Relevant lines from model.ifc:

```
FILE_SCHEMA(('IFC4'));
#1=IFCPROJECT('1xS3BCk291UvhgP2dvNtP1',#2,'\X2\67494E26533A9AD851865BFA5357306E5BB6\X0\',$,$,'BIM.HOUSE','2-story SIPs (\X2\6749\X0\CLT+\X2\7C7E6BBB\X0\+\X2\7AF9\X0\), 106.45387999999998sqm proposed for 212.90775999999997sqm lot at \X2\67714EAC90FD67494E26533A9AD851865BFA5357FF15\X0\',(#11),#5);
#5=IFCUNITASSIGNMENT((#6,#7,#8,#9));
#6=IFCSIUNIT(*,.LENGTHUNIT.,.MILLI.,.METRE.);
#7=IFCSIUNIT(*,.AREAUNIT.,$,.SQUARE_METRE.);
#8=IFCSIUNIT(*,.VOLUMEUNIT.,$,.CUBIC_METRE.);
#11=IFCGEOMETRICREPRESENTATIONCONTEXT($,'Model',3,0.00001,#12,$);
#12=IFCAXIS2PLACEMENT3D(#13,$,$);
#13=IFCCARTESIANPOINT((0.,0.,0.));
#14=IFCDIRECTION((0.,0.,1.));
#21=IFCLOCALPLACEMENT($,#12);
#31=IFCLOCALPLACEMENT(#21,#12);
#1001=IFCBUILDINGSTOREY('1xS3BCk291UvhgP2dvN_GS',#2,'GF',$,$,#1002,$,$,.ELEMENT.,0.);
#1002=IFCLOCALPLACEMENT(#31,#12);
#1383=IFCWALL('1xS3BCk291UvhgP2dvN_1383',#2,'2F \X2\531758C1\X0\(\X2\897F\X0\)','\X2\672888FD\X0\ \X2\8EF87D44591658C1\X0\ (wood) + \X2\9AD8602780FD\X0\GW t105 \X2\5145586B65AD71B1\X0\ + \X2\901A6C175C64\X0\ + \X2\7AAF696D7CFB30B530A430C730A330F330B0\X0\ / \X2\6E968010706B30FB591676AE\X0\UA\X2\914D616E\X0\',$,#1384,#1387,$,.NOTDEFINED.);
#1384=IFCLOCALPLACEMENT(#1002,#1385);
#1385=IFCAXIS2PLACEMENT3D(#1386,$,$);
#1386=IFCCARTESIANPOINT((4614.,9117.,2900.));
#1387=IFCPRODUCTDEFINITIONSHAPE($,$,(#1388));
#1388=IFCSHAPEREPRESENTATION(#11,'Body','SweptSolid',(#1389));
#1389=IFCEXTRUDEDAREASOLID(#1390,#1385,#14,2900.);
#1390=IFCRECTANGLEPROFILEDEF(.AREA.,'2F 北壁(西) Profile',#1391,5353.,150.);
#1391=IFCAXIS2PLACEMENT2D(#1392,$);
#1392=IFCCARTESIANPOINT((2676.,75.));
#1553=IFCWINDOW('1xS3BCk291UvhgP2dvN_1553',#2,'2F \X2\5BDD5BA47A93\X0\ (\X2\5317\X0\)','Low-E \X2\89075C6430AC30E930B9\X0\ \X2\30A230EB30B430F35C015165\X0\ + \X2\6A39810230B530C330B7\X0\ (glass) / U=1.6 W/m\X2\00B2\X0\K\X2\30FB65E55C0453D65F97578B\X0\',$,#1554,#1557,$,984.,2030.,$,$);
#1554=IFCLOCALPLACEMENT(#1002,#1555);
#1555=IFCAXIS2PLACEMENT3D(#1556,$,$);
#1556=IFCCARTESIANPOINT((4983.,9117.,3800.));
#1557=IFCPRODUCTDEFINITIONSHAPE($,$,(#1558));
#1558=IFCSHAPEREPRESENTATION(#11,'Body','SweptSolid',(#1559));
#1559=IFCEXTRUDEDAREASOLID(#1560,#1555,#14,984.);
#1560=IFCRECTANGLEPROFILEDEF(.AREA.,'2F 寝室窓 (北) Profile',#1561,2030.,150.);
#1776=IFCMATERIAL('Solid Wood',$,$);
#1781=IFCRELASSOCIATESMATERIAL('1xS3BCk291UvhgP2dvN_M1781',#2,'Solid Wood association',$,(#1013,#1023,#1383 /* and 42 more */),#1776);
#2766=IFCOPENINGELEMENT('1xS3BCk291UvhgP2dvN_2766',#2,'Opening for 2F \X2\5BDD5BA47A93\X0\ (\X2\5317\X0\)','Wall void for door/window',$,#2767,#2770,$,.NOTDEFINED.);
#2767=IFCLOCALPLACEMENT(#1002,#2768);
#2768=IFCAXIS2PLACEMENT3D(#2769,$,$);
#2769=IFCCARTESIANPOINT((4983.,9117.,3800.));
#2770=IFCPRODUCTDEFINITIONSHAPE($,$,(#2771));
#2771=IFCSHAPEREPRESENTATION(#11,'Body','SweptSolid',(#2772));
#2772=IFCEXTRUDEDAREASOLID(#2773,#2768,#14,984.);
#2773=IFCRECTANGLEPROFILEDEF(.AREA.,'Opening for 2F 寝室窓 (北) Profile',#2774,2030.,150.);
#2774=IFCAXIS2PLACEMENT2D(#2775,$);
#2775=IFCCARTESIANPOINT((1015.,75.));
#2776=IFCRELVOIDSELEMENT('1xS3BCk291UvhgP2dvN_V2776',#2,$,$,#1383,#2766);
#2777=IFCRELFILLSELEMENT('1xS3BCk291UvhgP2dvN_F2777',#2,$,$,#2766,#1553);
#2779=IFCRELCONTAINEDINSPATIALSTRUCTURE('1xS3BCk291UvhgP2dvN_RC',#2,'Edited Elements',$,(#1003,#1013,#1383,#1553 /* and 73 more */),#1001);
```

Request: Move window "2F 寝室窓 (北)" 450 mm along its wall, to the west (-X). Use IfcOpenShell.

```python
import ifcopenshell
import ifcopenshell.api.geometry
import ifcopenshell.util.placement
import ifcopenshell.util.unit

model = ifcopenshell.open("model.ifc")
unit_scale = ifcopenshell.util.unit.calculate_unit_scale(model)

window = model.by_guid("1xS3BCk291UvhgP2dvN_1553")
opening = window.FillsVoids[0].RelatingOpeningElement
wall = opening.VoidsElements[0].RelatingBuildingElement

wall_matrix = ifcopenshell.util.placement.get_local_placement(wall.ObjectPlacement)
shift = wall_matrix[:3, 0] * -0.45 / unit_scale
before = ifcopenshell.util.placement.get_local_placement(window.ObjectPlacement)[:3, 3].copy()

# The window is not placed relative to its opening, so move both.
for product in (opening, window):
    matrix = ifcopenshell.util.placement.get_local_placement(product.ObjectPlacement)
    matrix[:3, 3] += shift
    ifcopenshell.api.geometry.edit_object_placement(model, product=product, matrix=matrix, is_si=False)

after = ifcopenshell.util.placement.get_local_placement(window.ObjectPlacement)[:3, 3]
print("window moved by", (after - before).round(3) + 0.0)

model.write("model_rev.ifc")
```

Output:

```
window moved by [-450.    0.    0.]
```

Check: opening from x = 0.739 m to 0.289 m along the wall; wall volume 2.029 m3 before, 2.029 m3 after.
